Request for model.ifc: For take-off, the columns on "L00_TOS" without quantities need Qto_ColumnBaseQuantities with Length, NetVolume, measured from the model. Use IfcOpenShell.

First a look at what the model holds.

```python
import ifcopenshell
import ifcopenshell.util.element
import ifcopenshell.util.unit

model = ifcopenshell.open("model.ifc")
print(model.schema)
for unit_type in ("LENGTHUNIT", "AREAUNIT", "VOLUMEUNIT"):
    print(unit_type, ifcopenshell.util.unit.calculate_unit_scale(model, unit_type))
storey = next(s for s in model.by_type("IfcBuildingStorey") if s.Name == "L00_TOS")
columns = [e for e in ifcopenshell.util.element.get_decomposition(storey) if e.is_a("IfcColumn")]
for e in sorted(columns, key=lambda e: e.id()):
    print(e.id(), e.is_a(), e.Name, list(ifcopenshell.util.element.get_psets(e, qtos_only=True)), sep=" | ")
```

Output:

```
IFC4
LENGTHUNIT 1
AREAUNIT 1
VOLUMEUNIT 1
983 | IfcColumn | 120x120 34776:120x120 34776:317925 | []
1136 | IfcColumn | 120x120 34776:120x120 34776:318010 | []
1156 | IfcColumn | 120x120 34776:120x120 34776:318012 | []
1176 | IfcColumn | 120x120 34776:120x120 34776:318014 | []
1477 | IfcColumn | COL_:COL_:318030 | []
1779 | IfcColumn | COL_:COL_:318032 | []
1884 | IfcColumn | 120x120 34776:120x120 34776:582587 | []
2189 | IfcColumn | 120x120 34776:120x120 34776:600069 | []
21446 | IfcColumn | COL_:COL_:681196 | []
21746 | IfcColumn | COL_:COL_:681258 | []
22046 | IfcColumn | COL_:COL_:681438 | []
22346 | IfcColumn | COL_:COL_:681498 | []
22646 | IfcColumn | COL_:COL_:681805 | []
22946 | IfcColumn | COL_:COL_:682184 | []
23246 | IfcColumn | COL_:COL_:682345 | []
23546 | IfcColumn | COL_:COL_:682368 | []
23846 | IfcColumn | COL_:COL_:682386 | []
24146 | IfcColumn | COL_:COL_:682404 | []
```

```python
import ifcopenshell
import ifcopenshell.api.pset
import ifcopenshell.geom
import ifcopenshell.util.element
import ifcopenshell.util.shape
import ifcopenshell.util.unit

model = ifcopenshell.open("model.ifc")
unit_scale = ifcopenshell.util.unit.calculate_unit_scale(model)
volume_scale = ifcopenshell.util.unit.calculate_unit_scale(model, "VOLUMEUNIT")
settings = ifcopenshell.geom.settings()

storey = next(s for s in model.by_type("IfcBuildingStorey") if s.Name == "L00_TOS")
columns = [e for e in ifcopenshell.util.element.get_decomposition(storey) if e.is_a("IfcColumn")]

for e in sorted(columns, key=lambda e: e.id()):
    if ifcopenshell.util.element.get_psets(e, qtos_only=True, should_inherit=False):
        continue
    # Geometry comes back in metres, in the element's own axes.
    shape = ifcopenshell.geom.create_shape(settings, e)
    values = {
        "Length": ifcopenshell.util.shape.get_z(shape.geometry) / unit_scale,
        "NetVolume": ifcopenshell.util.shape.get_volume(shape.geometry) / volume_scale,
    }
    qto = ifcopenshell.api.pset.add_qto(model, product=e, name="Qto_ColumnBaseQuantities")
    ifcopenshell.api.pset.edit_qto(model, qto=qto, properties=values)
    print(e.id(), {k: round(v, 3) for k, v in values.items()})

model.write("model_updated.ifc")
```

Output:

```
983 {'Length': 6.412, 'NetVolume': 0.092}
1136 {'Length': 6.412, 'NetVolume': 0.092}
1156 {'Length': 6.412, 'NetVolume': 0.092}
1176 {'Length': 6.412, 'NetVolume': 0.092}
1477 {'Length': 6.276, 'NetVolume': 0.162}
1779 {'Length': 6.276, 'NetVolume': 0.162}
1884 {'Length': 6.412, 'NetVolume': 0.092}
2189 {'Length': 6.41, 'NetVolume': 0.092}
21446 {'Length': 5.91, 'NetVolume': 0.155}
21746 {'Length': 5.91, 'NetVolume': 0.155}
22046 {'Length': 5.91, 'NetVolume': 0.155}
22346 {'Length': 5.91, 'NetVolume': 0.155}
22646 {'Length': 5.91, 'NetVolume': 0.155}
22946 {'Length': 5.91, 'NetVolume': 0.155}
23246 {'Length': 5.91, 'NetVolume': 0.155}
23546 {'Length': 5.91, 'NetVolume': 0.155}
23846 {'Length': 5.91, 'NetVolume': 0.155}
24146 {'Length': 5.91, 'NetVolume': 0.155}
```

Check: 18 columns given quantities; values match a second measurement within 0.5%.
